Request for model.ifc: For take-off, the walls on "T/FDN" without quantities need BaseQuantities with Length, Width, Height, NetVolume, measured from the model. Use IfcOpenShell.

First a look at what the model holds.

```python
import ifcopenshell
import ifcopenshell.util.element
import ifcopenshell.util.unit

model = ifcopenshell.open("model.ifc")
print(model.schema)
for unit_type in ("LENGTHUNIT", "AREAUNIT", "VOLUMEUNIT"):
    print(unit_type, ifcopenshell.util.unit.calculate_unit_scale(model, unit_type))
storey = next(s for s in model.by_type("IfcBuildingStorey") if s.Name == "T/FDN")
walls = [e for e in ifcopenshell.util.element.get_decomposition(storey) if e.is_a("IfcWall")]
for e in sorted(walls, key=lambda e: e.id()):
    print(e.id(), e.is_a(), e.Name, list(ifcopenshell.util.element.get_psets(e, qtos_only=True)), sep=" | ")
```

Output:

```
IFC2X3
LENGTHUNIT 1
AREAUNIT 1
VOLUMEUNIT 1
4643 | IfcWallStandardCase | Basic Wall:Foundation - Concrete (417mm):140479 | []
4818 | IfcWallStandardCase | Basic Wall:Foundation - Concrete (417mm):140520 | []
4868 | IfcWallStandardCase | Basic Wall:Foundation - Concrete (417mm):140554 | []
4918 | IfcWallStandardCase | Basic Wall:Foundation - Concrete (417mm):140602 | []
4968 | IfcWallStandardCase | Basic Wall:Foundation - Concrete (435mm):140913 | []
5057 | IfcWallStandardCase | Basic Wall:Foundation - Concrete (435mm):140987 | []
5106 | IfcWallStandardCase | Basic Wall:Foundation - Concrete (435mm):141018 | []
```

```python
import ifcopenshell
import ifcopenshell.api.pset
import ifcopenshell.geom
import ifcopenshell.util.element
import ifcopenshell.util.shape
import ifcopenshell.util.unit

model = ifcopenshell.open("model.ifc")
unit_scale = ifcopenshell.util.unit.calculate_unit_scale(model)
volume_scale = ifcopenshell.util.unit.calculate_unit_scale(model, "VOLUMEUNIT")
settings = ifcopenshell.geom.settings()

storey = next(s for s in model.by_type("IfcBuildingStorey") if s.Name == "T/FDN")
walls = [e for e in ifcopenshell.util.element.get_decomposition(storey) if e.is_a("IfcWall")]

for e in sorted(walls, key=lambda e: e.id()):
    if ifcopenshell.util.element.get_psets(e, qtos_only=True, should_inherit=False):
        continue
    # Geometry comes back in metres, in the element's own axes.
    shape = ifcopenshell.geom.create_shape(settings, e)
    values = {
        "Length": ifcopenshell.util.shape.get_x(shape.geometry) / unit_scale,
        "Width": ifcopenshell.util.shape.get_y(shape.geometry) / unit_scale,
        "Height": ifcopenshell.util.shape.get_z(shape.geometry) / unit_scale,
        "NetVolume": ifcopenshell.util.shape.get_volume(shape.geometry) / volume_scale,
    }
    qto = ifcopenshell.api.pset.add_qto(model, product=e, name="BaseQuantities")
    ifcopenshell.api.pset.edit_qto(model, qto=qto, properties=values)
    print(e.id(), {k: round(v, 3) for k, v in values.items()})

model.write("model_updated.ifc")
```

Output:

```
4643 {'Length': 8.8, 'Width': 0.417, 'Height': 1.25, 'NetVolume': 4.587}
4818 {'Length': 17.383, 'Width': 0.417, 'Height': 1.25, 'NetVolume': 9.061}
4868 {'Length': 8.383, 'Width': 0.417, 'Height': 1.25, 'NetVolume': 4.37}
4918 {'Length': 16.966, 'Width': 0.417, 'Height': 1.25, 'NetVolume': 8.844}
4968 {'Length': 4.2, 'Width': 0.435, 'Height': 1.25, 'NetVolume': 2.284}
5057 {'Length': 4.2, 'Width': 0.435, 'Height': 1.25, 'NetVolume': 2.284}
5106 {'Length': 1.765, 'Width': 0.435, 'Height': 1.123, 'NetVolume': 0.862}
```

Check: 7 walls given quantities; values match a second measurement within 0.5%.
